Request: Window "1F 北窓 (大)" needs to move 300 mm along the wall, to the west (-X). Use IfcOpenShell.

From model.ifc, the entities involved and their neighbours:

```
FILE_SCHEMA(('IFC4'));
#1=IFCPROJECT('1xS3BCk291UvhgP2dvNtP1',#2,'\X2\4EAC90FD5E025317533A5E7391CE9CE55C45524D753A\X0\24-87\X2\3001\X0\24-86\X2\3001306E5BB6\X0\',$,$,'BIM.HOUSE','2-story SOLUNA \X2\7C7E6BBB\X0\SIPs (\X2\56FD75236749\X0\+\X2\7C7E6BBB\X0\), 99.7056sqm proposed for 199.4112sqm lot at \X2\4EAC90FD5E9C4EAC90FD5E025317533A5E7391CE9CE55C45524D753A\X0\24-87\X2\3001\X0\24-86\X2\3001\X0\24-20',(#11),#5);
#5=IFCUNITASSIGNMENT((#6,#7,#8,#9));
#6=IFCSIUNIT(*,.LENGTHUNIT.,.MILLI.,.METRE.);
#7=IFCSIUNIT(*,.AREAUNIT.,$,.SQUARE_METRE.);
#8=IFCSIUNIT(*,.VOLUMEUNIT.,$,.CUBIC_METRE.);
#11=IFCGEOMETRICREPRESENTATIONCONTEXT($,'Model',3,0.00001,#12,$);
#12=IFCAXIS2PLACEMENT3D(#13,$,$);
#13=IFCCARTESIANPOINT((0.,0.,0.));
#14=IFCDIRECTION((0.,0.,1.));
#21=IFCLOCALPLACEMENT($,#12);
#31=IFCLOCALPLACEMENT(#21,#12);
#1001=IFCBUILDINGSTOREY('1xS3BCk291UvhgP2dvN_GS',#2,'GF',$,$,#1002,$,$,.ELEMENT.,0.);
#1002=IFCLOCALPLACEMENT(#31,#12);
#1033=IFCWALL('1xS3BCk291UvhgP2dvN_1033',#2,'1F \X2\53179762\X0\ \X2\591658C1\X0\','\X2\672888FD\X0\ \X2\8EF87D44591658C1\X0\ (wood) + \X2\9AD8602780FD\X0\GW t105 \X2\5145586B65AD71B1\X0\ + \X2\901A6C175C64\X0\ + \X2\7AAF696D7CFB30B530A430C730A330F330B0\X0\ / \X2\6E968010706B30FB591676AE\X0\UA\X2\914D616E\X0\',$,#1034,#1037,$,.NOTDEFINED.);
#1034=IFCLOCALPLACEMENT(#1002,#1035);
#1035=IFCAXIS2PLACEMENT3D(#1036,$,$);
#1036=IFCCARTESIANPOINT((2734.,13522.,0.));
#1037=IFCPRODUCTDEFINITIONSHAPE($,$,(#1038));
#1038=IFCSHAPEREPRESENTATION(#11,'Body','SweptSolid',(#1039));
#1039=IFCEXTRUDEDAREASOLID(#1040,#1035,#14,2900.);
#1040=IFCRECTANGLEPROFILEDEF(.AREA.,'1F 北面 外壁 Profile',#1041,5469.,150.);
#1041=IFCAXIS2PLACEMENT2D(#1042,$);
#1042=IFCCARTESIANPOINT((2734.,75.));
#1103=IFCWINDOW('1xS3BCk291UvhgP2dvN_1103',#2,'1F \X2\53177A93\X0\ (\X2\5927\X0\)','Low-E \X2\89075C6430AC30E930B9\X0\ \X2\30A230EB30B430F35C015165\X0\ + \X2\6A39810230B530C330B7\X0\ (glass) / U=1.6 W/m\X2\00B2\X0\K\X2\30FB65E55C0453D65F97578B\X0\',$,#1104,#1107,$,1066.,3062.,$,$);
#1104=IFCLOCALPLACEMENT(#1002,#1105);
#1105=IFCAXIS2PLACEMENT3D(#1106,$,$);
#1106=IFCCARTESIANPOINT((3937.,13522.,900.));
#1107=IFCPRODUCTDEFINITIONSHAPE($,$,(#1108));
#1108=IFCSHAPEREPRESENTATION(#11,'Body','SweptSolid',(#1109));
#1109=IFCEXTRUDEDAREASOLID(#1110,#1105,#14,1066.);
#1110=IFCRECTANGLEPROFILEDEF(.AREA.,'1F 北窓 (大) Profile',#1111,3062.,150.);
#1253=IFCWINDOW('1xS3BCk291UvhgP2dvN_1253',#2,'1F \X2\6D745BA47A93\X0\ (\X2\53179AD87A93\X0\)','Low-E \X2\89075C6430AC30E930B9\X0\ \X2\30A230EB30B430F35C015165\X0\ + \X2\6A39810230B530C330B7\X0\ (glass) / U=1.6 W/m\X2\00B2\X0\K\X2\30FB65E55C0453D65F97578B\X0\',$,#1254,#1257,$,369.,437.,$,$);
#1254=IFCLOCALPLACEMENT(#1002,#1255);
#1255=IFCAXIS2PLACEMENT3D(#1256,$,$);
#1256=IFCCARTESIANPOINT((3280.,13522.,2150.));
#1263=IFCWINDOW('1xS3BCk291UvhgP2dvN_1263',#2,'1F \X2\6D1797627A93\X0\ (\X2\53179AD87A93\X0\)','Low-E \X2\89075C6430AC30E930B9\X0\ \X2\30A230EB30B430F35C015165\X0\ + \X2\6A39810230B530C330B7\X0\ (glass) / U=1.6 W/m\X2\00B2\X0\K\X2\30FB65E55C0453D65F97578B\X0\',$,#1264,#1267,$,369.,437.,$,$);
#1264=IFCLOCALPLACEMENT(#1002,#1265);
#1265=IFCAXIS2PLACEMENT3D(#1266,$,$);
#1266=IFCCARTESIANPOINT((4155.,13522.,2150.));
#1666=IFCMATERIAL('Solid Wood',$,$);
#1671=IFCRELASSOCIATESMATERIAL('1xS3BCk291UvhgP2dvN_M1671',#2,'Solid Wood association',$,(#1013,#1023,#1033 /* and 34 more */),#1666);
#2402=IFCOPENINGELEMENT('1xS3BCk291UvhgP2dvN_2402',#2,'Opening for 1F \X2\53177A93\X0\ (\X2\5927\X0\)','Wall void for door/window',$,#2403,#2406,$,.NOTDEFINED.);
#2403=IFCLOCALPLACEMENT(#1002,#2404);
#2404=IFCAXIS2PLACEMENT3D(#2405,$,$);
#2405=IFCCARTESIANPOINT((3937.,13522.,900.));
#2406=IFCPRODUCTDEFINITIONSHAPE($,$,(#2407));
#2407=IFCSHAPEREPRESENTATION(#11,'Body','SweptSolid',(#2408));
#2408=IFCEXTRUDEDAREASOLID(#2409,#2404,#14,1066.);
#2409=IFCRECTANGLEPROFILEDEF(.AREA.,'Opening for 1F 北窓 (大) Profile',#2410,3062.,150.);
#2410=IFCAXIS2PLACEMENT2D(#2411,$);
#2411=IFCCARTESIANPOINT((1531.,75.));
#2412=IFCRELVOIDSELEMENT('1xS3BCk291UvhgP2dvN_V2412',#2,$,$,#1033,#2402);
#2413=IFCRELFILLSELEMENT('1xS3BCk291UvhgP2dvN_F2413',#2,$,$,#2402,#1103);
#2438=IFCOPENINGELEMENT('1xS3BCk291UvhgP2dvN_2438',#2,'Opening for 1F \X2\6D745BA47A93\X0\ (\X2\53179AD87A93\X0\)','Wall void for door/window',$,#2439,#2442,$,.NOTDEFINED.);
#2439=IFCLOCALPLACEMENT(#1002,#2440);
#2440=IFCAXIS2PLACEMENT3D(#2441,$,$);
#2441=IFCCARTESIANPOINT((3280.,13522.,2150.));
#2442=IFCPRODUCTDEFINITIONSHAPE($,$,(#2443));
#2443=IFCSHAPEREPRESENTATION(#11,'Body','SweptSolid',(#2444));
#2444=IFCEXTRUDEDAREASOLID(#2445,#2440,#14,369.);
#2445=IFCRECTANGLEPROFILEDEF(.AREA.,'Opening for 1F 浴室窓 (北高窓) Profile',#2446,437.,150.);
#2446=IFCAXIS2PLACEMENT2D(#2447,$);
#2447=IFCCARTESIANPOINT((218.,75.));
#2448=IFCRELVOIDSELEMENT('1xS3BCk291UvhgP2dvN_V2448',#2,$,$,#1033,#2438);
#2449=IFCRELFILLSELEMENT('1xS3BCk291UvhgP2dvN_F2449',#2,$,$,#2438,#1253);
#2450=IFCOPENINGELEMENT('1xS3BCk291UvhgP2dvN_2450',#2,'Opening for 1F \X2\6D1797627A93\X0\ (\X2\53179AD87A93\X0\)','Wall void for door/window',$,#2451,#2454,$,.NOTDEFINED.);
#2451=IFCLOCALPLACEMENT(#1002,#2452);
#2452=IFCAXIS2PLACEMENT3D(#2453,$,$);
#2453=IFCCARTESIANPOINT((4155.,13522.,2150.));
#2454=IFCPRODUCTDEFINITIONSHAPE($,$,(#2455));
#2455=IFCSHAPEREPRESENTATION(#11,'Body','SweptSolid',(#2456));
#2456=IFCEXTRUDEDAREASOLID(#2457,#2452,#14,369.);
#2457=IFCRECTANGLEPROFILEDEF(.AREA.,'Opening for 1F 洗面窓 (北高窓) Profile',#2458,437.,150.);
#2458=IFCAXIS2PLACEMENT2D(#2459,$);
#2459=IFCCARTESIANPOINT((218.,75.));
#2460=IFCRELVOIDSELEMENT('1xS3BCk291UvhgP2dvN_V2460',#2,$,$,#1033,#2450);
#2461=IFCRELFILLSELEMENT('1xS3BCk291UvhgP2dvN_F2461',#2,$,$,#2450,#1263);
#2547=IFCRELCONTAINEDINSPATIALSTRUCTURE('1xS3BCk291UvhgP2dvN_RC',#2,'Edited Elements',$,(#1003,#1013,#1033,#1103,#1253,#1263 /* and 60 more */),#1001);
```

```python
import ifcopenshell
import ifcopenshell.api.geometry
import ifcopenshell.util.placement
import ifcopenshell.util.unit

model = ifcopenshell.open("model.ifc")
unit_scale = ifcopenshell.util.unit.calculate_unit_scale(model)

window = model.by_guid("1xS3BCk291UvhgP2dvN_1103")
opening = window.FillsVoids[0].RelatingOpeningElement
wall = opening.VoidsElements[0].RelatingBuildingElement

wall_matrix = ifcopenshell.util.placement.get_local_placement(wall.ObjectPlacement)
shift = wall_matrix[:3, 0] * -0.3 / unit_scale
before = ifcopenshell.util.placement.get_local_placement(window.ObjectPlacement)[:3, 3].copy()

# The window is not placed relative to its opening, so move both.
for product in (opening, window):
    matrix = ifcopenshell.util.placement.get_local_placement(product.ObjectPlacement)
    matrix[:3, 3] += shift
    ifcopenshell.api.geometry.edit_object_placement(model, product=product, matrix=matrix, is_si=False)

after = ifcopenshell.util.placement.get_local_placement(window.ObjectPlacement)[:3, 3]
print("window moved by", (after - before).round(3) + 0.0)

model.write("model_v2.ifc")
```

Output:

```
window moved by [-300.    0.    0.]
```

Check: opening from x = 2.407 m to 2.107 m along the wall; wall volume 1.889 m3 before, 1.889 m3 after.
